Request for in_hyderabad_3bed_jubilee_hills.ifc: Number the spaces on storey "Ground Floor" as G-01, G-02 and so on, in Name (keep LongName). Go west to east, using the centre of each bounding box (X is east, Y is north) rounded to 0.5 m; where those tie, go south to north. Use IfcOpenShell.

First a look at what the model holds.

```python
import ifcopenshell
import ifcopenshell.util.element
import ifcopenshell.util.placement

model = ifcopenshell.open("in_hyderabad_3bed_jubilee_hills.ifc")
print(model.schema)
storey = next(s for s in model.by_type("IfcBuildingStorey") if s.Name == "Ground Floor")
spaces = [e for e in ifcopenshell.util.element.get_decomposition(storey) if e.is_a("IfcSpace")]
for e in sorted(spaces, key=lambda e: e.id()):
    origin = ifcopenshell.util.placement.get_local_placement(e.ObjectPlacement)[:3, 3]
    print(e.id(), e.Name, e.LongName, origin.round(2) + 0.0, sep=" | ")
```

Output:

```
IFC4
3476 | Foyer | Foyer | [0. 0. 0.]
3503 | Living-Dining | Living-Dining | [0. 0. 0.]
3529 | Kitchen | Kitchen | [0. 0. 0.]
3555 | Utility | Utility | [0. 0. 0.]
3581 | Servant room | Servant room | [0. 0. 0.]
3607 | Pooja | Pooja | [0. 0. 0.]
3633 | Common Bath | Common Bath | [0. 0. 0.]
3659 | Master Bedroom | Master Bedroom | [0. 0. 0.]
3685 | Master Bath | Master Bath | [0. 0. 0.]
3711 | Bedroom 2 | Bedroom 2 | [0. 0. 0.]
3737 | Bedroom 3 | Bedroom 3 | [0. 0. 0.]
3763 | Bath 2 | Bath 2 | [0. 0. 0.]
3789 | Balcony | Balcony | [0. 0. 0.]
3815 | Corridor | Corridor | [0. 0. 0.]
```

```python
import ifcopenshell
import ifcopenshell.geom
import ifcopenshell.util.element
import ifcopenshell.util.shape

model = ifcopenshell.open("in_hyderabad_3bed_jubilee_hills.ifc")
settings = ifcopenshell.geom.settings()
settings.set("use-world-coords", True)


def centre(element):
    shape = ifcopenshell.geom.create_shape(settings, element)
    return ifcopenshell.util.shape.get_bbox_centroid(shape.geometry)


storey = next(s for s in model.by_type("IfcBuildingStorey") if s.Name == "Ground Floor")
spaces = [e for e in ifcopenshell.util.element.get_decomposition(storey) if e.is_a("IfcSpace")]

# Insertion points can sit at a corner or the storey origin, so sort by the geometry (in metres).
centres = {e: centre(e) for e in spaces}
spaces.sort(key=lambda e: (round(centres[e][0] / 0.5), centres[e][1]))

for i, e in enumerate(spaces, start=1):
    number = f"G-{i:02d}"
    e.Name = number
    print(e.id(), number)

model.write("in_hyderabad_3bed_jubilee_hills-out.ifc")
```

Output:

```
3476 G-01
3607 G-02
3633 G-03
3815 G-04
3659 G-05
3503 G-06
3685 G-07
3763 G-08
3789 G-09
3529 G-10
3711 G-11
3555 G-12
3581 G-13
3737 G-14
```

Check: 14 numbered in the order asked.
